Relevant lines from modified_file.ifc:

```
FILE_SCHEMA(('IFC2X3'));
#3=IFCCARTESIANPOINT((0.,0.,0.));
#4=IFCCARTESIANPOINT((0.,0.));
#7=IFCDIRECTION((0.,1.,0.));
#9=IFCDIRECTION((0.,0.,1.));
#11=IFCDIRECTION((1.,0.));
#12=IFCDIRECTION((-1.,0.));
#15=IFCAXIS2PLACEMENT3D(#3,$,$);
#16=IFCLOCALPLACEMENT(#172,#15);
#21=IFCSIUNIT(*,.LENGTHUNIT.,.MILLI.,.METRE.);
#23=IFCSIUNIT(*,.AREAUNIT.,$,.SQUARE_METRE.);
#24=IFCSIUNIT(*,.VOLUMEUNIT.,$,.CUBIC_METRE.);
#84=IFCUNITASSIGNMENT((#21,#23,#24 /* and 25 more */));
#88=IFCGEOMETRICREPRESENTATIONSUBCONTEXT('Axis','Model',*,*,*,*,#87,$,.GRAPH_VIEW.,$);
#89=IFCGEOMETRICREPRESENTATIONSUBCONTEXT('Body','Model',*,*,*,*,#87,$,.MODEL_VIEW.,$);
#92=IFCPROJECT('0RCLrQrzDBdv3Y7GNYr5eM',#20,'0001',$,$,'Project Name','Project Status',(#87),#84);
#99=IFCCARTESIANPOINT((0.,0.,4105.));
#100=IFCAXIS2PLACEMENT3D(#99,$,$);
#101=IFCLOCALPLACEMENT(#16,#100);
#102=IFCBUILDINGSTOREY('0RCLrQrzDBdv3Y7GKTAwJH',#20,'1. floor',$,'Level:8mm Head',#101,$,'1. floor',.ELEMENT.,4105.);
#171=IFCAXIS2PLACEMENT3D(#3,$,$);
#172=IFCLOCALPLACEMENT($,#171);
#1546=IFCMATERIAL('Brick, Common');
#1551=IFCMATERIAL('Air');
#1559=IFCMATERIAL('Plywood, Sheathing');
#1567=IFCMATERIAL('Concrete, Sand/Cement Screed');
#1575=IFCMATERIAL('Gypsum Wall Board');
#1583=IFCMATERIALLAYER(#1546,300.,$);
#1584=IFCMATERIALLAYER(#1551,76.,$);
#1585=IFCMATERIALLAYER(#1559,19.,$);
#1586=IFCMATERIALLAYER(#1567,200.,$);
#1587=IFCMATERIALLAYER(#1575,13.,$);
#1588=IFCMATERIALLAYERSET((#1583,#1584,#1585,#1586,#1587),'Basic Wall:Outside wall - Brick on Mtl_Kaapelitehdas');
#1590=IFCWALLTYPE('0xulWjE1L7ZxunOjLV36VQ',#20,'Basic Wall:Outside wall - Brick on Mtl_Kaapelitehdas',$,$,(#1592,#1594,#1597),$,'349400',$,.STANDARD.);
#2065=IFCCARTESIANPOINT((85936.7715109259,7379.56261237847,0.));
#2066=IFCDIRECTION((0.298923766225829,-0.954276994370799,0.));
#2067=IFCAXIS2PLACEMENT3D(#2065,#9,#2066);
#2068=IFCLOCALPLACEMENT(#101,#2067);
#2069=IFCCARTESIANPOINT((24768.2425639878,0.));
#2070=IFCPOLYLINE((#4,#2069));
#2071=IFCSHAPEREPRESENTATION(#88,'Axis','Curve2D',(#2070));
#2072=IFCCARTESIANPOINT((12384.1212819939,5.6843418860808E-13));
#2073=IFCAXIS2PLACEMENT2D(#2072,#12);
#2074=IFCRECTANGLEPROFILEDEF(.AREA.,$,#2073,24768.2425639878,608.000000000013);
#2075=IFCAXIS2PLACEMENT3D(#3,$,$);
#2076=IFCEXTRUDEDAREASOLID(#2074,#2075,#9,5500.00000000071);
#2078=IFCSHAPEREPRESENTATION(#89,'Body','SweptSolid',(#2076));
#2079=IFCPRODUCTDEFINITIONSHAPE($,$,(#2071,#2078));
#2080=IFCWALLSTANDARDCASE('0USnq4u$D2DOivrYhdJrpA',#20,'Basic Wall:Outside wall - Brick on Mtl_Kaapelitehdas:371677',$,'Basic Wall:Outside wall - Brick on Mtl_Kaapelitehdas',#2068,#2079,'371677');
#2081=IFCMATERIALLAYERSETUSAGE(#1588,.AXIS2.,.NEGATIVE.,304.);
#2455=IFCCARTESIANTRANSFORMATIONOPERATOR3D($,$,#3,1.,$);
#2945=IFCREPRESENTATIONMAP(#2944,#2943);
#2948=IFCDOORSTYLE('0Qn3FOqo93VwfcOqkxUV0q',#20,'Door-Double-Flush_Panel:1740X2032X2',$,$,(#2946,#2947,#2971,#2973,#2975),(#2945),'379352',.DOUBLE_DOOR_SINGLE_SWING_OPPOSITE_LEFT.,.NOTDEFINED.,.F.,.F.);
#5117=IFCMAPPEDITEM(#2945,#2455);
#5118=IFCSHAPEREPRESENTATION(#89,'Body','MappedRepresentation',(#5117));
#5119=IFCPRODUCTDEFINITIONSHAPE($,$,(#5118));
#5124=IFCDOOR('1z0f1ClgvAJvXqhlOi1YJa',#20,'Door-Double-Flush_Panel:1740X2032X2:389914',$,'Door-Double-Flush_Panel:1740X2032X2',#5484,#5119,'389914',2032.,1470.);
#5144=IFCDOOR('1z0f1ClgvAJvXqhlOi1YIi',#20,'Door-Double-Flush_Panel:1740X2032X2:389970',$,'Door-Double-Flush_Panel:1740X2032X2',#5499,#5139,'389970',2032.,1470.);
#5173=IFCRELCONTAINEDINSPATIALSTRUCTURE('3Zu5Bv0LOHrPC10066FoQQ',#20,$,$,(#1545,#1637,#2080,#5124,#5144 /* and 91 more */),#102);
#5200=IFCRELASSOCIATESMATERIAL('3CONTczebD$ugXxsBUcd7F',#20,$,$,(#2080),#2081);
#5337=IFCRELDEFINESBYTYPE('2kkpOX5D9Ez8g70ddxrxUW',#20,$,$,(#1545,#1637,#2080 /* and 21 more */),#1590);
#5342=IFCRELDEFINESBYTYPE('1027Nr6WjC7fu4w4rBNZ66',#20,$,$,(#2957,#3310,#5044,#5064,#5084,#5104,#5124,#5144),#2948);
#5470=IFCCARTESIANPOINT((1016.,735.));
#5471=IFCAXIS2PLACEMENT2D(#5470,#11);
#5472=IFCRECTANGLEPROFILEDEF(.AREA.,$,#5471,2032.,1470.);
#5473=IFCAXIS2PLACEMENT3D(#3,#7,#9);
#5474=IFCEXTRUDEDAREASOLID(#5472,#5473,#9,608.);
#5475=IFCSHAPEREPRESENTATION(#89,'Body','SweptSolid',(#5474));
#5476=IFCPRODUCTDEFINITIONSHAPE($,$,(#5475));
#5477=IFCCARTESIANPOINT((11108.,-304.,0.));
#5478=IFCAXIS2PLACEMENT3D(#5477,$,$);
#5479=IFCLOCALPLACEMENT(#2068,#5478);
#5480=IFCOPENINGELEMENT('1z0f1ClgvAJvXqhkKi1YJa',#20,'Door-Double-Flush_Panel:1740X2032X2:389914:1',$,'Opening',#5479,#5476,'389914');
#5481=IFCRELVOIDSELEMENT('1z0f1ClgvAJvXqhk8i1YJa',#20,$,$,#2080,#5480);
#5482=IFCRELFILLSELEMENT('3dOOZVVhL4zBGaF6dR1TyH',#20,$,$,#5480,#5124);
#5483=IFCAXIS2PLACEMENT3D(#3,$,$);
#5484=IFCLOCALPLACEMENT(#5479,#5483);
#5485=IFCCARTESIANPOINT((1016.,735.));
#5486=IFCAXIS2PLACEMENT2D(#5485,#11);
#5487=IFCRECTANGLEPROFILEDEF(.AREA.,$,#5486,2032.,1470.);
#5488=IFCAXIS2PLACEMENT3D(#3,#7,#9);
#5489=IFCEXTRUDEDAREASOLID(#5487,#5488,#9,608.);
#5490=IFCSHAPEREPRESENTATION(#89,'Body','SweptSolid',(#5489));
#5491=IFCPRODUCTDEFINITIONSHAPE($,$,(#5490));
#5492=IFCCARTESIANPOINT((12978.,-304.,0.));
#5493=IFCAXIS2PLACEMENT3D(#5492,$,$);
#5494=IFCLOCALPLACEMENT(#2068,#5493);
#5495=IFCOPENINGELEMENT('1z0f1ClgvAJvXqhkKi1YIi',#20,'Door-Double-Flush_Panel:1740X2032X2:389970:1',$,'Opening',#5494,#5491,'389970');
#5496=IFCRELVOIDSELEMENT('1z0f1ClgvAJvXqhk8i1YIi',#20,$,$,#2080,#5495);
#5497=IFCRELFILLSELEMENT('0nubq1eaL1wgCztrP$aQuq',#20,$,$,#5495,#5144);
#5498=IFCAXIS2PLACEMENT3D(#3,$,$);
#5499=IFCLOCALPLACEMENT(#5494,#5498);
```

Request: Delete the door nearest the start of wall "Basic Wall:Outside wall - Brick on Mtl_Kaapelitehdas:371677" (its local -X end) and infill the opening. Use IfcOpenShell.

```python
import ifcopenshell
import ifcopenshell.api.feature
import ifcopenshell.api.root
import ifcopenshell.geom
import ifcopenshell.util.shape

model = ifcopenshell.open("modified_file.ifc")
settings = ifcopenshell.geom.settings()


def volume(element):
    """Net volume in cubic metres, openings subtracted."""
    shape = ifcopenshell.geom.create_shape(settings, element)
    return ifcopenshell.util.shape.get_volume(shape.geometry)


door = model.by_id(5124)
opening = door.FillsVoids[0].RelatingOpeningElement
wall = opening.VoidsElements[0].RelatingBuildingElement
before = volume(wall)

ifcopenshell.api.root.remove_product(model, product=door)
ifcopenshell.api.feature.remove_feature(model, feature=opening)

after = volume(wall)

print(f"wall volume {before:.3f} -> {after:.3f} m3")

model.write("modified_file_updated.ifc")
```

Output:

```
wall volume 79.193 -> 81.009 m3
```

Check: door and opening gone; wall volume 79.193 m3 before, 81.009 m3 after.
